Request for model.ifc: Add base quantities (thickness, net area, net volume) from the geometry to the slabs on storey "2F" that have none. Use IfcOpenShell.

First a look at what the model holds.

```python
import ifcopenshell
import ifcopenshell.util.element
import ifcopenshell.util.unit

model = ifcopenshell.open("model.ifc")
print(model.schema)
for unit_type in ("LENGTHUNIT", "AREAUNIT", "VOLUMEUNIT"):
    print(unit_type, ifcopenshell.util.unit.calculate_unit_scale(model, unit_type))
storey = next(s for s in model.by_type("IfcBuildingStorey") if s.Name == "2F")
slabs = [e for e in ifcopenshell.util.element.get_decomposition(storey) if e.is_a("IfcSlab")]
for e in sorted(slabs, key=lambda e: e.id()):
    print(e.id(), e.is_a(), e.Name, list(ifcopenshell.util.element.get_psets(e, qtos_only=True)), sep=" | ")
```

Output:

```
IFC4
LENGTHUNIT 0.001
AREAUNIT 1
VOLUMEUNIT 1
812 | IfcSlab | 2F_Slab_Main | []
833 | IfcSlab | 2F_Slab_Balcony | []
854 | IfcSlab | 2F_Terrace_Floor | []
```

```python
import ifcopenshell
import ifcopenshell.api.pset
import ifcopenshell.geom
import ifcopenshell.util.element
import ifcopenshell.util.shape
import ifcopenshell.util.unit

model = ifcopenshell.open("model.ifc")
unit_scale = ifcopenshell.util.unit.calculate_unit_scale(model)
area_scale = ifcopenshell.util.unit.calculate_unit_scale(model, "AREAUNIT")
volume_scale = ifcopenshell.util.unit.calculate_unit_scale(model, "VOLUMEUNIT")
settings = ifcopenshell.geom.settings()

storey = next(s for s in model.by_type("IfcBuildingStorey") if s.Name == "2F")
slabs = [e for e in ifcopenshell.util.element.get_decomposition(storey) if e.is_a("IfcSlab")]

for e in sorted(slabs, key=lambda e: e.id()):
    if ifcopenshell.util.element.get_psets(e, qtos_only=True, should_inherit=False):
        continue
    # Geometry comes back in metres, in the element's own axes.
    shape = ifcopenshell.geom.create_shape(settings, e)
    values = {
        "Width": ifcopenshell.util.shape.get_z(shape.geometry) / unit_scale,
        "NetArea": ifcopenshell.util.shape.get_footprint_area(shape.geometry) / area_scale,
        "NetVolume": ifcopenshell.util.shape.get_volume(shape.geometry) / volume_scale,
    }
    qto = ifcopenshell.api.pset.add_qto(model, product=e, name="Qto_SlabBaseQuantities")
    ifcopenshell.api.pset.edit_qto(model, qto=qto, properties=values)
    print(e.id(), {k: round(v, 3) for k, v in values.items()})

model.write("model_edited.ifc")
```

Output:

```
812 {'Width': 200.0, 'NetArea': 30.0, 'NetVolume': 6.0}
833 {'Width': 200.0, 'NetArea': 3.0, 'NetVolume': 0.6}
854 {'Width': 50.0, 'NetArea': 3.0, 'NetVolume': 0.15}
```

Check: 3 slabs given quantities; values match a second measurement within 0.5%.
